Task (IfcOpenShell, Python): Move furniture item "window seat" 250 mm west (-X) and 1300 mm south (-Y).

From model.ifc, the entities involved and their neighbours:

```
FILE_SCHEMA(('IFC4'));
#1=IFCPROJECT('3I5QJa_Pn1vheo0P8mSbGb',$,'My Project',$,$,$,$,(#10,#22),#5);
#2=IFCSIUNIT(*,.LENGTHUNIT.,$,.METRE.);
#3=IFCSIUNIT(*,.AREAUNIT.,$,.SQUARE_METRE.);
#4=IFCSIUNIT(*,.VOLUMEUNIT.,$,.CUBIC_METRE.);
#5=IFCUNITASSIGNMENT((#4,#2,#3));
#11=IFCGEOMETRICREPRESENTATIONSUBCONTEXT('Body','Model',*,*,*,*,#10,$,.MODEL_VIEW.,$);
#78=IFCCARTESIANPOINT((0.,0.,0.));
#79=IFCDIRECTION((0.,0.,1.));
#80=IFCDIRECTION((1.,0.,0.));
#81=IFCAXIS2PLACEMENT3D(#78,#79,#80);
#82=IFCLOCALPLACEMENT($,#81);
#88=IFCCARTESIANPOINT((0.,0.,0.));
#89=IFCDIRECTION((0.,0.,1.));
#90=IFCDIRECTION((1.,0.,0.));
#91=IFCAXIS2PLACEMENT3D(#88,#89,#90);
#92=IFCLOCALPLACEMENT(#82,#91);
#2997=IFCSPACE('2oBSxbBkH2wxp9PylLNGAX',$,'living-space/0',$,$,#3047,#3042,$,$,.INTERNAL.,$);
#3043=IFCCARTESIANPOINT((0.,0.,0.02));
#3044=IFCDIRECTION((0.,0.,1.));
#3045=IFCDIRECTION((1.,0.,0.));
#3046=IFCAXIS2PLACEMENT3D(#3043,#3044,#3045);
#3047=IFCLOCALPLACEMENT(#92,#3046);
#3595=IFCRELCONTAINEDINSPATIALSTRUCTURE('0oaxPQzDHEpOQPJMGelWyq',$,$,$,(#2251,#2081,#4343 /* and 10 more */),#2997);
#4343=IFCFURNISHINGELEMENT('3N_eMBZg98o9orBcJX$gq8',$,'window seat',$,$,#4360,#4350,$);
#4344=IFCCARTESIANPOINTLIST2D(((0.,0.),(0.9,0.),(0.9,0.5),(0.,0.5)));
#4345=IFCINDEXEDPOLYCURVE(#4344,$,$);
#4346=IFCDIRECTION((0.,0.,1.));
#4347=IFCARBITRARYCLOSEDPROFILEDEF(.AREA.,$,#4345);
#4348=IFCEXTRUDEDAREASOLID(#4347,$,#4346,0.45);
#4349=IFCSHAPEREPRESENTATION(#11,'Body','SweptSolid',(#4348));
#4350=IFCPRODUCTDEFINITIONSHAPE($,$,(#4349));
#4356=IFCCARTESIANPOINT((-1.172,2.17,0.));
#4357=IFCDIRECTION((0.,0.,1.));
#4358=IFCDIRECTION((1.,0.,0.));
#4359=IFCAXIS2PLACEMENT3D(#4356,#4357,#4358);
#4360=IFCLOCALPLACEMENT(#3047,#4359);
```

```python
import ifcopenshell
import ifcopenshell.api.geometry
import ifcopenshell.util.placement

model = ifcopenshell.open("model.ifc")

item = model.by_id(4343)
matrix = ifcopenshell.util.placement.get_local_placement(item.ObjectPlacement)
matrix[0, 3] -= 0.25
matrix[1, 3] -= 1.3
ifcopenshell.api.geometry.edit_object_placement(model, product=item, matrix=matrix, is_si=False)

print(ifcopenshell.util.placement.get_local_placement(item.ObjectPlacement).round(3) + 0.0)

model.write("model_rev.ifc")
```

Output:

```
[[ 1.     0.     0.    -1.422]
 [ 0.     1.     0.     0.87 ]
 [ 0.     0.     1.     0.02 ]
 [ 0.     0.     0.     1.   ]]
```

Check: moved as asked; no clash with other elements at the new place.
